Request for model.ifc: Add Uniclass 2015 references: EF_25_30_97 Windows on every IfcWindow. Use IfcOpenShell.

First a look at what the model holds.

```python
import ifcopenshell

model = ifcopenshell.open("model.ifc")
print(model.schema)
print("classifications:", [c.Name for c in model.by_type("IfcClassification")])
for ifc_class in ("IfcDoor", "IfcRoof", "IfcStair", "IfcWall", "IfcWindow"):
    print(ifc_class, len(model.by_type(ifc_class)))
```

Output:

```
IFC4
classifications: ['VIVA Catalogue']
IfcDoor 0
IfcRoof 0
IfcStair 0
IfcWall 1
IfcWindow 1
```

```python
import ifcopenshell
import ifcopenshell.api.classification

model = ifcopenshell.open("model.ifc")

system = ifcopenshell.api.classification.add_classification(model, classification="Uniclass 2015")

codes = {
    "IfcWindow": ("EF_25_30_97", "Windows"),
}
for ifc_class, (code, name) in codes.items():
    products = model.by_type(ifc_class)
    ifcopenshell.api.classification.add_reference(
        model, products=products, classification=system, identification=code, name=name
    )
    print(code, len(products))

model.write("model-out.ifc")
```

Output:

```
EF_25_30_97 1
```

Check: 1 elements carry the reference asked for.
